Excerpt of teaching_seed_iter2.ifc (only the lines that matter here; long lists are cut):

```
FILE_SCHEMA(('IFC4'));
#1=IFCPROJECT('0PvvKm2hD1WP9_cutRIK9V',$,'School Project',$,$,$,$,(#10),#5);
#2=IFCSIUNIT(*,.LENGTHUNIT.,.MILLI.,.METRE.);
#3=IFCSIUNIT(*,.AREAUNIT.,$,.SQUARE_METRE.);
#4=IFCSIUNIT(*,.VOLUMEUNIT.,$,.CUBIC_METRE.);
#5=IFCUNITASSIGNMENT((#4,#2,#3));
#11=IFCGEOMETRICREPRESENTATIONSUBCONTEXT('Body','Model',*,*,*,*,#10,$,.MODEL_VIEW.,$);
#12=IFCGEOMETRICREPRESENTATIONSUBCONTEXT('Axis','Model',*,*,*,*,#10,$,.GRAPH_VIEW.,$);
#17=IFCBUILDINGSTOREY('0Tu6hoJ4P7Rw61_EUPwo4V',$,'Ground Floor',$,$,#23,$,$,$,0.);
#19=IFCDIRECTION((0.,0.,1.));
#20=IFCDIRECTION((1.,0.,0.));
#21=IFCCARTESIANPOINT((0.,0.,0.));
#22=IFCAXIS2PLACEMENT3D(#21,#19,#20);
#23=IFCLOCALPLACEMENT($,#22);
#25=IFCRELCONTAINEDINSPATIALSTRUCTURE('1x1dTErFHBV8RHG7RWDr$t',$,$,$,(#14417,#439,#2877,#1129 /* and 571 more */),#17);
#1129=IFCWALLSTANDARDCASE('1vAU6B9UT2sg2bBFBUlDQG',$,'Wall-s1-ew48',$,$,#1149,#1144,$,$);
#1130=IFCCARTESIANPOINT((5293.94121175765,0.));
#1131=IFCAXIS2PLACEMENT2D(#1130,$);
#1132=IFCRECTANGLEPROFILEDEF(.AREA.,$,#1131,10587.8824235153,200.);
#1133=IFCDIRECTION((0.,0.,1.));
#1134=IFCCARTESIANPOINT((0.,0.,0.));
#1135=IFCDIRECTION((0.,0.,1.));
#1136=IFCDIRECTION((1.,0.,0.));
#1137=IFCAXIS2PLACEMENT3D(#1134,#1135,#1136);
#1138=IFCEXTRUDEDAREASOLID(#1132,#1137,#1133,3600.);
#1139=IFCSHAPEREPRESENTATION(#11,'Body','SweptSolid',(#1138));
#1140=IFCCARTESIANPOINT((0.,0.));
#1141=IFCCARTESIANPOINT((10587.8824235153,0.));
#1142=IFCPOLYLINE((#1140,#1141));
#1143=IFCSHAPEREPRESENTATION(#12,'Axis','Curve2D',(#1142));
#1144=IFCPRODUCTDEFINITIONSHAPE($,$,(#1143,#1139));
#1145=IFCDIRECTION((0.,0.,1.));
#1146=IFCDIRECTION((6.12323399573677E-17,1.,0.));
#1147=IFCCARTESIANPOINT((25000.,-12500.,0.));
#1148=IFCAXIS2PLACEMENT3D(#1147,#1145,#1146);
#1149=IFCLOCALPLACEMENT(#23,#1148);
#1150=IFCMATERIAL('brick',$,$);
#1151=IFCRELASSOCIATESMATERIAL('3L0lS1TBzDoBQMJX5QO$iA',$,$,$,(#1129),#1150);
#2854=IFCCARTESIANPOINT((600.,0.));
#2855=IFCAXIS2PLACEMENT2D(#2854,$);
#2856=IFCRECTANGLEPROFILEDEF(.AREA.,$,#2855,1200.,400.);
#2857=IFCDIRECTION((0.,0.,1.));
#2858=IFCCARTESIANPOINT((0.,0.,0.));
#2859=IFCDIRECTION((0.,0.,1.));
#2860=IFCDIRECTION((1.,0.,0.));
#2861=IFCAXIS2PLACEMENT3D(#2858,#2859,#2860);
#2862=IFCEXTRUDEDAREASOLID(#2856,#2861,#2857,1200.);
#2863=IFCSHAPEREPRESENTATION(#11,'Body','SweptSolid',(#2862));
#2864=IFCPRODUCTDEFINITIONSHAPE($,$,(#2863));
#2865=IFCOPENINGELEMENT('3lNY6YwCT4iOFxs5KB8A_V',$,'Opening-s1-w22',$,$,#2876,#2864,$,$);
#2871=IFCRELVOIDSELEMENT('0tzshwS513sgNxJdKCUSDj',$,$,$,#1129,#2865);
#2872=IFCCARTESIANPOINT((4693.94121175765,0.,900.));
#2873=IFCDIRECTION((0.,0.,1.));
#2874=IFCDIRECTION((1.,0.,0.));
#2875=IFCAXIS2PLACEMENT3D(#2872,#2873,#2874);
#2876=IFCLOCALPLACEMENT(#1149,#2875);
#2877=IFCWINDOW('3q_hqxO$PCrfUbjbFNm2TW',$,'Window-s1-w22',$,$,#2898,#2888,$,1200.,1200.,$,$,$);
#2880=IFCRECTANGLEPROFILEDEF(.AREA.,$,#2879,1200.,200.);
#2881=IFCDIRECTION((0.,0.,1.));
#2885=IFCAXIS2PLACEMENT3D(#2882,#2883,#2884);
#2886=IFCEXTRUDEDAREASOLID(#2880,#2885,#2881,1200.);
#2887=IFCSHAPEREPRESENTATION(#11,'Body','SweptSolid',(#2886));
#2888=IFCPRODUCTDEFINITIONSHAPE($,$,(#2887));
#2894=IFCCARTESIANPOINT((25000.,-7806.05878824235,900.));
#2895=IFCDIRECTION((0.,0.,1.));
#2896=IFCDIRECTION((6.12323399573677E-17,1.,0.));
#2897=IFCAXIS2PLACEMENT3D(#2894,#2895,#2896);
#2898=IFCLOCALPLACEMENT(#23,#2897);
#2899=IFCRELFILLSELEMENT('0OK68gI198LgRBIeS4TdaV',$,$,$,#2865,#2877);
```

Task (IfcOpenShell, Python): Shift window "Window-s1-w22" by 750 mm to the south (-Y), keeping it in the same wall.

```python
import ifcopenshell
import ifcopenshell.api.geometry
import ifcopenshell.util.placement
import ifcopenshell.util.unit

model = ifcopenshell.open("teaching_seed_iter2.ifc")
unit_scale = ifcopenshell.util.unit.calculate_unit_scale(model)

window = model.by_id(2877)
opening = window.FillsVoids[0].RelatingOpeningElement
wall = opening.VoidsElements[0].RelatingBuildingElement

wall_matrix = ifcopenshell.util.placement.get_local_placement(wall.ObjectPlacement)
shift = wall_matrix[:3, 0] * -0.75 / unit_scale
before = ifcopenshell.util.placement.get_local_placement(window.ObjectPlacement)[:3, 3].copy()

# The window is not placed relative to its opening, so move both.
for product in (opening, window):
    matrix = ifcopenshell.util.placement.get_local_placement(product.ObjectPlacement)
    matrix[:3, 3] += shift
    ifcopenshell.api.geometry.edit_object_placement(model, product=product, matrix=matrix, is_si=False)

after = ifcopenshell.util.placement.get_local_placement(window.ObjectPlacement)[:3, 3]
print("window moved by", (after - before).round(3) + 0.0)

model.write("teaching_seed_iter2_rev.ifc")
```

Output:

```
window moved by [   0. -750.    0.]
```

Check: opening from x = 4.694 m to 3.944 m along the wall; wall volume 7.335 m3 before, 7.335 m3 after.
